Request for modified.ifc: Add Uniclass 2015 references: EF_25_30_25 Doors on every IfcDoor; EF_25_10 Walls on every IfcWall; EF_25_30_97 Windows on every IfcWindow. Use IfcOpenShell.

First a look at what the model holds.

```python
import ifcopenshell

model = ifcopenshell.open("modified.ifc")
print(model.schema)
print("classifications:", [c.Name for c in model.by_type("IfcClassification")])
for ifc_class in ("IfcDoor", "IfcRoof", "IfcStair", "IfcWall", "IfcWindow"):
    print(ifc_class, len(model.by_type(ifc_class)))
```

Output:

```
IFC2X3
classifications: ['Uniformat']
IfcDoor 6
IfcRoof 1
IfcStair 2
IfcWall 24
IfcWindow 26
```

```python
import ifcopenshell
import ifcopenshell.api.classification

model = ifcopenshell.open("modified.ifc")

# IFC2X3 requires Source and Edition and has no link from the project to the system.
system = model.create_entity("IfcClassification", Source="NBS", Edition="2015", Name="Uniclass 2015")

codes = {
    "IfcDoor": ("EF_25_30_25", "Doors"),
    "IfcWall": ("EF_25_10", "Walls"),
    "IfcWindow": ("EF_25_30_97", "Windows"),
}
for ifc_class, (code, name) in codes.items():
    products = model.by_type(ifc_class)
    ifcopenshell.api.classification.add_reference(
        model, products=products, classification=system, identification=code, name=name
    )
    print(code, len(products))

model.write("modified_rev.ifc")
```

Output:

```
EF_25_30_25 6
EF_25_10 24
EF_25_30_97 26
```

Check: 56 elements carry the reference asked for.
